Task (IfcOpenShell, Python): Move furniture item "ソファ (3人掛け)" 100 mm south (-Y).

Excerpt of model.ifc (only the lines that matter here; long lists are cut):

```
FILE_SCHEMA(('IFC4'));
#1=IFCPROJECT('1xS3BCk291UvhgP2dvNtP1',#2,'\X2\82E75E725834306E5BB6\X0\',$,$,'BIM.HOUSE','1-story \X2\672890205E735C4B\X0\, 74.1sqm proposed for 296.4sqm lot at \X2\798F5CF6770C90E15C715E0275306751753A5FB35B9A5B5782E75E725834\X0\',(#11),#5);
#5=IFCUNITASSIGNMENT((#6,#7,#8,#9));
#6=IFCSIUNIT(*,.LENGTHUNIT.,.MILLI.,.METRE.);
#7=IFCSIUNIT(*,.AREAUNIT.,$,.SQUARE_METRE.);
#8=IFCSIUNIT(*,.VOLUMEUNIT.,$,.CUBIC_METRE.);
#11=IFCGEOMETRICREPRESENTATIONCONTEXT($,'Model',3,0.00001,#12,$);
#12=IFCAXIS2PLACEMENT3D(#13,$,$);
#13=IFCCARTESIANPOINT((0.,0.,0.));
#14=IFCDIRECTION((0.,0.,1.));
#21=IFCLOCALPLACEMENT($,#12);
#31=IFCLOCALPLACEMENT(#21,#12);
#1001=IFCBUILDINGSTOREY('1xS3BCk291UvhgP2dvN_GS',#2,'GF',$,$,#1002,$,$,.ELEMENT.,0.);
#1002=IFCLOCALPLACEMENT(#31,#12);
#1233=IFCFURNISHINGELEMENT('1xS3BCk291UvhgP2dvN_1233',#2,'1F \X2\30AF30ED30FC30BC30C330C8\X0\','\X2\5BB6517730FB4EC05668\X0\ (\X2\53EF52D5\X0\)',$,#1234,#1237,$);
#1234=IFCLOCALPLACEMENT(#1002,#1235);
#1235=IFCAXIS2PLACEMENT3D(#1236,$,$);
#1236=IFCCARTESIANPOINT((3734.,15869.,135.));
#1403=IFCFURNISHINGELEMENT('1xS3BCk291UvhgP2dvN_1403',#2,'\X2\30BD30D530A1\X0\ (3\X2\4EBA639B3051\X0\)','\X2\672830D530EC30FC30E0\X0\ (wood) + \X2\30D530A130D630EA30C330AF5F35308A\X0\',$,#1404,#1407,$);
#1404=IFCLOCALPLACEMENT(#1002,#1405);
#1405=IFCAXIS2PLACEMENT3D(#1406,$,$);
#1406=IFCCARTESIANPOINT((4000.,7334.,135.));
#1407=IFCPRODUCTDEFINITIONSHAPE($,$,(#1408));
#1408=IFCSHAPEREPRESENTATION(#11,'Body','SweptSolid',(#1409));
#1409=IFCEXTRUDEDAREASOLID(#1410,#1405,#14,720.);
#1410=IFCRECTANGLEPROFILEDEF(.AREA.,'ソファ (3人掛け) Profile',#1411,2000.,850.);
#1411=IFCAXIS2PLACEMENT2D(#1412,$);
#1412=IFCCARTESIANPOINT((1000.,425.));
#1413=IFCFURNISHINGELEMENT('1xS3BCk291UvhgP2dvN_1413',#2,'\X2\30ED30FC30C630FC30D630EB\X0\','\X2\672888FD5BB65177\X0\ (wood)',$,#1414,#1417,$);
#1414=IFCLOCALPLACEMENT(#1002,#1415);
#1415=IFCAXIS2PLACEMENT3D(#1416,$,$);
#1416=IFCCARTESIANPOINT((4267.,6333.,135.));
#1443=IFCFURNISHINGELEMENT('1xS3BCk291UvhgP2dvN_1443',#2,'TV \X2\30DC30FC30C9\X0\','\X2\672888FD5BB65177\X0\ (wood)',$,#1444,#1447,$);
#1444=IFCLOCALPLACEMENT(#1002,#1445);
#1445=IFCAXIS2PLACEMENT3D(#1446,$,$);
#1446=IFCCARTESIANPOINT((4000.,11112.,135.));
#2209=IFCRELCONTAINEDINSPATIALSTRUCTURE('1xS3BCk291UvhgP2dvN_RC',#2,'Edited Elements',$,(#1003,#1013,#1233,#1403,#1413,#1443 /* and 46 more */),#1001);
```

```python
import ifcopenshell
import ifcopenshell.api.geometry
import ifcopenshell.util.placement
import ifcopenshell.util.unit

model = ifcopenshell.open("model.ifc")
unit_scale = ifcopenshell.util.unit.calculate_unit_scale(model)

item = model.by_guid("1xS3BCk291UvhgP2dvN_1403")
matrix = ifcopenshell.util.placement.get_local_placement(item.ObjectPlacement)
matrix[1, 3] -= 0.1 / unit_scale
ifcopenshell.api.geometry.edit_object_placement(model, product=item, matrix=matrix, is_si=False)

print(ifcopenshell.util.placement.get_local_placement(item.ObjectPlacement).round(3) + 0.0)

model.write("model_updated.ifc")
```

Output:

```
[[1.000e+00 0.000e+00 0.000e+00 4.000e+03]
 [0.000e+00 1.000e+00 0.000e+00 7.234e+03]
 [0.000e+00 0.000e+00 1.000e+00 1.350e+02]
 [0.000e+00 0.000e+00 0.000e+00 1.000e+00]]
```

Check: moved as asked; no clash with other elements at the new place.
